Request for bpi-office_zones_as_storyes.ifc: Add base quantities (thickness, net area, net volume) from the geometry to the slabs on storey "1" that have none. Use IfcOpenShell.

First a look at what the model holds.

```python
import ifcopenshell
import ifcopenshell.util.element
import ifcopenshell.util.unit

model = ifcopenshell.open("bpi-office_zones_as_storyes.ifc")
print(model.schema)
for unit_type in ("LENGTHUNIT", "AREAUNIT", "VOLUMEUNIT"):
    print(unit_type, ifcopenshell.util.unit.calculate_unit_scale(model, unit_type))
storey = next(s for s in model.by_type("IfcBuildingStorey") if s.Name == "1")
slabs = [e for e in ifcopenshell.util.element.get_decomposition(storey) if e.is_a("IfcSlab")]
for e in sorted(slabs, key=lambda e: e.id()):
    print(e.id(), e.is_a(), e.Name, list(ifcopenshell.util.element.get_psets(e, qtos_only=True)), sep=" | ")
```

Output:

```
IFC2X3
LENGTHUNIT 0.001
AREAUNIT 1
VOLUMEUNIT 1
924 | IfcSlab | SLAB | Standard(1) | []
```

```python
import ifcopenshell
import ifcopenshell.api.pset
import ifcopenshell.geom
import ifcopenshell.util.element
import ifcopenshell.util.shape
import ifcopenshell.util.unit

model = ifcopenshell.open("bpi-office_zones_as_storyes.ifc")
unit_scale = ifcopenshell.util.unit.calculate_unit_scale(model)
area_scale = ifcopenshell.util.unit.calculate_unit_scale(model, "AREAUNIT")
volume_scale = ifcopenshell.util.unit.calculate_unit_scale(model, "VOLUMEUNIT")
settings = ifcopenshell.geom.settings()

storey = next(s for s in model.by_type("IfcBuildingStorey") if s.Name == "1")
slabs = [e for e in ifcopenshell.util.element.get_decomposition(storey) if e.is_a("IfcSlab")]

for e in sorted(slabs, key=lambda e: e.id()):
    if ifcopenshell.util.element.get_psets(e, qtos_only=True, should_inherit=False):
        continue
    # Geometry comes back in metres, in the element's own axes.
    shape = ifcopenshell.geom.create_shape(settings, e)
    values = {
        "Width": ifcopenshell.util.shape.get_z(shape.geometry) / unit_scale,
        "NetArea": ifcopenshell.util.shape.get_footprint_area(shape.geometry) / area_scale,
        "NetVolume": ifcopenshell.util.shape.get_volume(shape.geometry) / volume_scale,
    }
    qto = ifcopenshell.api.pset.add_qto(model, product=e, name="BaseQuantities")
    ifcopenshell.api.pset.edit_qto(model, qto=qto, properties=values)
    print(e.id(), {k: round(v, 3) for k, v in values.items()})

model.write("bpi-office_zones_as_storyes_edited.ifc")
```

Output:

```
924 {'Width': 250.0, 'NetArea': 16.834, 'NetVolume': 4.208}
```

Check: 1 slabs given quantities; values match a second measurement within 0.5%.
